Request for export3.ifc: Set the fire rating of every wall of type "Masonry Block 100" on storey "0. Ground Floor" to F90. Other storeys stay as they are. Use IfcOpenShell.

First a look at what the model holds.

```python
import ifcopenshell
import ifcopenshell.util.element

model = ifcopenshell.open("export3.ifc")
print(model.schema)
storey = next(s for s in model.by_type("IfcBuildingStorey") if s.Name == "0. Ground Floor")
walls = [e for e in ifcopenshell.util.element.get_decomposition(storey) if e.is_a("IfcWall")]
seen = {}
for e in walls:
    element_type = ifcopenshell.util.element.get_type(e)
    key = (element_type.Name if element_type != e and element_type else None, ifcopenshell.util.element.get_pset(e, "Pset_WallCommon", "FireRating"))
    seen[key] = seen.get(key, 0) + 1
for (name, value), count in sorted(seen.items(), key=str):
    print(count, "x", name, "|", value)
```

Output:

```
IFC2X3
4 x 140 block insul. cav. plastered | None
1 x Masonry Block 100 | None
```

```python
import ifcopenshell
import ifcopenshell.api.pset
import ifcopenshell.util.element

model = ifcopenshell.open("export3.ifc")

storey = next(s for s in model.by_type("IfcBuildingStorey") if s.Name == "0. Ground Floor")
walls = [e for e in ifcopenshell.util.element.get_decomposition(storey) if e.is_a("IfcWall")]

count = 0
for e in walls:
    element_type = ifcopenshell.util.element.get_type(e)
    if element_type in (None, e) or element_type.Name != "Masonry Block 100":
        continue
    # add_pset returns the element's existing set when there is one.
    pset = ifcopenshell.api.pset.add_pset(model, product=e, name="Pset_WallCommon")
    ifcopenshell.api.pset.edit_pset(model, pset=pset, properties={"FireRating": "F90"})
    count += 1

print(count, "walls updated")

model.write("export3_updated.ifc")
```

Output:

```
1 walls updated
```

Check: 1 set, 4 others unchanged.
